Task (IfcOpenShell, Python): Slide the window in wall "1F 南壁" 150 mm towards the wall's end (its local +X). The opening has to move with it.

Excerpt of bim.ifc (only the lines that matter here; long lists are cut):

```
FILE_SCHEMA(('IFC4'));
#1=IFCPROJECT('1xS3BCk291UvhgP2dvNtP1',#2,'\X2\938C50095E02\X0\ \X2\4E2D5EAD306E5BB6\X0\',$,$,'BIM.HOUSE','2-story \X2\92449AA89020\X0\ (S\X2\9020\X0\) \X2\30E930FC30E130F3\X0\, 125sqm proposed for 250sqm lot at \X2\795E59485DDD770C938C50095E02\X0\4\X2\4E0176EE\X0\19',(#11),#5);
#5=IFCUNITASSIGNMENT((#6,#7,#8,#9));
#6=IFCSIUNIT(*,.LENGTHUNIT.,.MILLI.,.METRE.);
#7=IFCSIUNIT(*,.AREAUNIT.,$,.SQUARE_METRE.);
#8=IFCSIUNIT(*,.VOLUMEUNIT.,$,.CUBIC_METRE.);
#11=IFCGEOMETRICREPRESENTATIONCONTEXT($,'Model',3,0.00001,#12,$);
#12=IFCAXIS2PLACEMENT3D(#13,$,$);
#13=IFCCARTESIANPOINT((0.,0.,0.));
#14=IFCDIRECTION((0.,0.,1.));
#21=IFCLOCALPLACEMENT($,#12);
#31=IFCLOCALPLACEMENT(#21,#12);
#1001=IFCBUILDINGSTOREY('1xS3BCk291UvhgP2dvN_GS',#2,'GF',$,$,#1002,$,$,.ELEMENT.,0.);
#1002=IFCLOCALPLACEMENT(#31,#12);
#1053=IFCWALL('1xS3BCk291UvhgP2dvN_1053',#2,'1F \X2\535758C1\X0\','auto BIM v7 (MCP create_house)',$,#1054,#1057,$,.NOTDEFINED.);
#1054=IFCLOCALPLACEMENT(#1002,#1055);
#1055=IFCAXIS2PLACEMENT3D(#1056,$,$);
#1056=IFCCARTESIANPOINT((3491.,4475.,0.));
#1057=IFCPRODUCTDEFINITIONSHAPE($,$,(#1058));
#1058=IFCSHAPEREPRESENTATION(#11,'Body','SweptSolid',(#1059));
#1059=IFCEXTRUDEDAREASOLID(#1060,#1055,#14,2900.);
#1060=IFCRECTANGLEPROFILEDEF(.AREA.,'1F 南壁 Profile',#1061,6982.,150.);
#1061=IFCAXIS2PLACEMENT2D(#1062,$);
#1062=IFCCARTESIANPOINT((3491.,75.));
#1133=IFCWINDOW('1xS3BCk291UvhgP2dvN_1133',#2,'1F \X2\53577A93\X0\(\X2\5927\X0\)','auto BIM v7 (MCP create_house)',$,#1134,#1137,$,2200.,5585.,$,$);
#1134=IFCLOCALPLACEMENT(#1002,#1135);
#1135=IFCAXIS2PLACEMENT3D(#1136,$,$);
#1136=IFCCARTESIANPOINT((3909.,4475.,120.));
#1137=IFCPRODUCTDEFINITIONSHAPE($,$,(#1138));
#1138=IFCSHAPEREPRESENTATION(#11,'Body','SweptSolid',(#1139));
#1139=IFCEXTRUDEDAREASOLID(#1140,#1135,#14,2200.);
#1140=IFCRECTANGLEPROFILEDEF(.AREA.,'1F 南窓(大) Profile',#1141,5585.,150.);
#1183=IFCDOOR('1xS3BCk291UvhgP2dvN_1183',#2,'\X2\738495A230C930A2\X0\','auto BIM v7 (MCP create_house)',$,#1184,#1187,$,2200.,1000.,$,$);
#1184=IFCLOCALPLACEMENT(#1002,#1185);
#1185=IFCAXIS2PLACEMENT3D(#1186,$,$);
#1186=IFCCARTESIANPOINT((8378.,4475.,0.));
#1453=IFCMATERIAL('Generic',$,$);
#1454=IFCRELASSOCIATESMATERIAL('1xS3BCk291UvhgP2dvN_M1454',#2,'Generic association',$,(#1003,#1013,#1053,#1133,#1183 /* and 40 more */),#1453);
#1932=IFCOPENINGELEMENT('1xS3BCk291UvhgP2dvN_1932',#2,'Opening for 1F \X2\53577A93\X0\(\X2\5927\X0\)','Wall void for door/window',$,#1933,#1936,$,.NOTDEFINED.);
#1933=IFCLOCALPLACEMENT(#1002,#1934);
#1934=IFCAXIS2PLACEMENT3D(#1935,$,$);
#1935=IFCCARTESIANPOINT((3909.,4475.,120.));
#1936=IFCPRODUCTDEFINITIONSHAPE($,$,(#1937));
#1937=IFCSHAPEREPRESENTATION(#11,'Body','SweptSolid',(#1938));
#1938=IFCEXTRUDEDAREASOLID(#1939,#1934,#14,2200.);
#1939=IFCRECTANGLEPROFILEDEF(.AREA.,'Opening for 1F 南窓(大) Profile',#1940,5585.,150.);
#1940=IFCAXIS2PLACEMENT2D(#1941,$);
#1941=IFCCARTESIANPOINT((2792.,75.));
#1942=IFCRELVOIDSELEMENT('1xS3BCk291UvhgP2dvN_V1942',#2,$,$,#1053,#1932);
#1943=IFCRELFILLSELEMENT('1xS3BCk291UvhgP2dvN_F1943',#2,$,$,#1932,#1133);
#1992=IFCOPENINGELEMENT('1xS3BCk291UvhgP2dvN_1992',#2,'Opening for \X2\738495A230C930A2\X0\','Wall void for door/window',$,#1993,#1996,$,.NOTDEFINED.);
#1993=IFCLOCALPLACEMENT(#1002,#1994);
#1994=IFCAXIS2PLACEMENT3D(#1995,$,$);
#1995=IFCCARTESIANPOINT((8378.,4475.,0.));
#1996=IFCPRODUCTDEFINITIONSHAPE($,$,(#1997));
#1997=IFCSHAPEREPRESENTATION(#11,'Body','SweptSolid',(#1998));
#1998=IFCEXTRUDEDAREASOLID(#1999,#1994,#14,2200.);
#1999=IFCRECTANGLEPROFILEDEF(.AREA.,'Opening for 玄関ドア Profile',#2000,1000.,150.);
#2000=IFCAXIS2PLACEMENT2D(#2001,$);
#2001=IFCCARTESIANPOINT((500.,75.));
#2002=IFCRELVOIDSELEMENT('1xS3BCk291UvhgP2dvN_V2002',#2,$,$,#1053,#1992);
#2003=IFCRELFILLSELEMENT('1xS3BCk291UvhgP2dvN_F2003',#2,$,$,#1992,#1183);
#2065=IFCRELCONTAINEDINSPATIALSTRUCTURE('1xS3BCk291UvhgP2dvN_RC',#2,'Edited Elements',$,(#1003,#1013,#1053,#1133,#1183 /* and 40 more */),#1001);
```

```python
import ifcopenshell
import ifcopenshell.api.geometry
import ifcopenshell.util.placement
import ifcopenshell.util.unit

model = ifcopenshell.open("bim.ifc")
unit_scale = ifcopenshell.util.unit.calculate_unit_scale(model)

window = model.by_guid("1xS3BCk291UvhgP2dvN_1133")
opening = window.FillsVoids[0].RelatingOpeningElement
wall = opening.VoidsElements[0].RelatingBuildingElement

wall_matrix = ifcopenshell.util.placement.get_local_placement(wall.ObjectPlacement)
shift = wall_matrix[:3, 0] * 0.15 / unit_scale
before = ifcopenshell.util.placement.get_local_placement(window.ObjectPlacement)[:3, 3].copy()

# The window is not placed relative to its opening, so move both.
for product in (opening, window):
    matrix = ifcopenshell.util.placement.get_local_placement(product.ObjectPlacement)
    matrix[:3, 3] += shift
    ifcopenshell.api.geometry.edit_object_placement(model, product=product, matrix=matrix, is_si=False)

after = ifcopenshell.util.placement.get_local_placement(window.ObjectPlacement)[:3, 3]
print("window moved by", (after - before).round(3) + 0.0)

model.write("bim_edited.ifc")
```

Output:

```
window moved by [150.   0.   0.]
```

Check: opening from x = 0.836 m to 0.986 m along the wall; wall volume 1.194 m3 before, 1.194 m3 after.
